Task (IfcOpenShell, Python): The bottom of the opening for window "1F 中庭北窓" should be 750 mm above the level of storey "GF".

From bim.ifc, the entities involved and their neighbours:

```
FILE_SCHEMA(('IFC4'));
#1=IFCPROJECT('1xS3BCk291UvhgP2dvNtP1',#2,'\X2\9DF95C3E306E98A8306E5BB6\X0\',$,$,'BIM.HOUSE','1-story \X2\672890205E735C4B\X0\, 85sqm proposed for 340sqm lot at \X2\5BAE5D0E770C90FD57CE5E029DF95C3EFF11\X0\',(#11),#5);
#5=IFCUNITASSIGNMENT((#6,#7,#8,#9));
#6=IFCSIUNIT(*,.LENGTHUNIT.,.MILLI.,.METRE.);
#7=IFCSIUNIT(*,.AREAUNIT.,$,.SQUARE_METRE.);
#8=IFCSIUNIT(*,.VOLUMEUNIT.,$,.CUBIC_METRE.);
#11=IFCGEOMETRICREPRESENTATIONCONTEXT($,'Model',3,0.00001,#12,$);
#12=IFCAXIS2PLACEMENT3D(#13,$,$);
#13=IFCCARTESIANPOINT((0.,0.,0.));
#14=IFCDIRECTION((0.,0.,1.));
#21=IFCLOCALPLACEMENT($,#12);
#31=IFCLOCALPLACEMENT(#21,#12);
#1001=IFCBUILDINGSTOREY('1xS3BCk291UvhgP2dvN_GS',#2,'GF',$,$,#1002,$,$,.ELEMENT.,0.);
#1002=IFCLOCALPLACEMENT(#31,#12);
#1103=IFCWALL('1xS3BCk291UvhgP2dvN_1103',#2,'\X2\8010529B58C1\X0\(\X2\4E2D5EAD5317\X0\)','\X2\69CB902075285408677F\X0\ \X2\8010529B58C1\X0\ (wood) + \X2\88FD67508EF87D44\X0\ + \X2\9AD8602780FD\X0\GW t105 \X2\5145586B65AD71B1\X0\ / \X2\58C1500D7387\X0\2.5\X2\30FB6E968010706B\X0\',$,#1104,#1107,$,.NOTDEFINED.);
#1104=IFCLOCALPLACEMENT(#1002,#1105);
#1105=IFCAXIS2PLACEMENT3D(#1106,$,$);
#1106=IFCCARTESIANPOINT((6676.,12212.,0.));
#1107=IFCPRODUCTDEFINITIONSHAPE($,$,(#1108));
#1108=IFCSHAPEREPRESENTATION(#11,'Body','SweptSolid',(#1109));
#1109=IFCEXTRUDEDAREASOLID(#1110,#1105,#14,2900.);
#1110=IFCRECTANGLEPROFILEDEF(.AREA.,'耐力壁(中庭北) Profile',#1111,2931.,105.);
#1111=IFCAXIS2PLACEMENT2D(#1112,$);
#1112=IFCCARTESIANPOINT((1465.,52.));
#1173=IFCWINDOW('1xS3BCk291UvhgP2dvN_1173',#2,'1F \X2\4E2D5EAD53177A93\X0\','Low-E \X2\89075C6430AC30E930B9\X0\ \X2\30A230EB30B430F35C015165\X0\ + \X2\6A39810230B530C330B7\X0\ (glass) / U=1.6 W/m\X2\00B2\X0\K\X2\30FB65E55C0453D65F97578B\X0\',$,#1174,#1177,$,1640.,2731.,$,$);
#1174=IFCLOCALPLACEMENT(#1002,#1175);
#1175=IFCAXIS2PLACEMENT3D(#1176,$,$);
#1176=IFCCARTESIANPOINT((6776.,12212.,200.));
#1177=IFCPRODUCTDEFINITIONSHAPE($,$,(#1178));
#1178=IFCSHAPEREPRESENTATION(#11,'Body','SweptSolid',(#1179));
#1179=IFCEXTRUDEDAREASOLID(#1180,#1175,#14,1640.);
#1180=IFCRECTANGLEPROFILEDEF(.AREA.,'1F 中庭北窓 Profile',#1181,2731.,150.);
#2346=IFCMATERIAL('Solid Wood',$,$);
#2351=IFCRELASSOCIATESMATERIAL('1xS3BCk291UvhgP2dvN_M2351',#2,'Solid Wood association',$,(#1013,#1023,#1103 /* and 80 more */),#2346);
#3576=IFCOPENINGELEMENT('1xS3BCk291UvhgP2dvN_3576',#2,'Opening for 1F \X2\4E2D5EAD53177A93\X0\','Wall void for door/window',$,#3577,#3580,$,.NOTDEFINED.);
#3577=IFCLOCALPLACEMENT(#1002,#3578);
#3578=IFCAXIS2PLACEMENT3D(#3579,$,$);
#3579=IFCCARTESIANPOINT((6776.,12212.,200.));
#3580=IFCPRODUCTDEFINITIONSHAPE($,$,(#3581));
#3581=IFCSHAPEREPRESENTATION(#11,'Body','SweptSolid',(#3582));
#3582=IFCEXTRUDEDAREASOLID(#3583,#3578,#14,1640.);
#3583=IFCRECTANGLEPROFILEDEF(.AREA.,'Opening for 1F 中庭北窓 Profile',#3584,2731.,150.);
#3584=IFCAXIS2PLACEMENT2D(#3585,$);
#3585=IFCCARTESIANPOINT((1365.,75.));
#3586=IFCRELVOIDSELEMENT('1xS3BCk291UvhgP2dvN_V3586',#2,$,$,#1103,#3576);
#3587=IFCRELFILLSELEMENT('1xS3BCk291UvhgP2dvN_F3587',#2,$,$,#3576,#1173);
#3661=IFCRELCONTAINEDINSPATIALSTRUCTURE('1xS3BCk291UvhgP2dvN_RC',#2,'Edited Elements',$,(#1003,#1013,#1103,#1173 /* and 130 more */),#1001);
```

```python
import numpy as np
import ifcopenshell
import ifcopenshell.api.geometry
import ifcopenshell.geom
import ifcopenshell.util.element
import ifcopenshell.util.placement
import ifcopenshell.util.shape
import ifcopenshell.util.unit

model = ifcopenshell.open("bim.ifc")
unit_scale = ifcopenshell.util.unit.calculate_unit_scale(model)

window = model.by_guid("1xS3BCk291UvhgP2dvN_1173")
opening = window.FillsVoids[0].RelatingOpeningElement
storey = ifcopenshell.util.element.get_container(window, ifc_class="IfcBuildingStorey")
level = ifcopenshell.util.placement.get_local_placement(storey.ObjectPlacement)[2, 3]

# The opening's origin need not be at the sill, so measure its lowest point.
shape = ifcopenshell.geom.create_shape(ifcopenshell.geom.settings(), opening)
bottom = ifcopenshell.util.shape.get_shape_bottom_elevation(shape, shape.geometry) / unit_scale
dz = level + 750.0 - bottom

shift = np.array([0.0, 0.0, dz])
# The window is not placed relative to its opening, so move both.
for product in (opening, window):
    matrix = ifcopenshell.util.placement.get_local_placement(product.ObjectPlacement)
    matrix[:3, 3] += shift
    ifcopenshell.api.geometry.edit_object_placement(model, product=product, matrix=matrix, is_si=False)

print(f"moved by {dz * unit_scale:+.3f} m")

model.write("bim_updated.ifc")
```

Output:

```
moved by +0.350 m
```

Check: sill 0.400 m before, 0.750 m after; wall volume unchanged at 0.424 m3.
